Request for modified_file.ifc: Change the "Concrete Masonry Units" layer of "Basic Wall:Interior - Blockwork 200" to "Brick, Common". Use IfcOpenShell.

First a look at what the model holds.

```python
import ifcopenshell
import ifcopenshell.util.element

model = ifcopenshell.open("modified_file.ifc")
print(model.schema)
for layer_set in model.by_type("IfcMaterialLayerSet"):
    if layer_set.LayerSetName == "Basic Wall:Interior - Blockwork 200":
        for layer in layer_set.MaterialLayers:
            print(layer.id(), layer.Material and layer.Material.Name, layer.LayerThickness, sep=" | ")
        print(len(ifcopenshell.util.element.get_elements_by_material(model, layer_set)), "elements and types use it")
print(sorted(m.Name for m in model.by_type("IfcMaterial") if m.Name)[:60])
```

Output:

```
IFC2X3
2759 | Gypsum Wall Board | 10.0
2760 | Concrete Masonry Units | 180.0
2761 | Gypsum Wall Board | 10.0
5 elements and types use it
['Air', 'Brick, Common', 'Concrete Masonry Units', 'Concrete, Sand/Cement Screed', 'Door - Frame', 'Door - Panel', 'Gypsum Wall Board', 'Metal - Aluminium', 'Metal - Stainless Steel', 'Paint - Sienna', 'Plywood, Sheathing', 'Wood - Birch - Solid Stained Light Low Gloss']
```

```python
import ifcopenshell
import ifcopenshell.api.material

model = ifcopenshell.open("modified_file.ifc")

layer_set = next(s for s in model.by_type("IfcMaterialLayerSet") if s.LayerSetName == "Basic Wall:Interior - Blockwork 200")
layer = next(l for l in layer_set.MaterialLayers if l.Material and l.Material.Name == "Concrete Masonry Units")
material = next(m for m in model.by_type("IfcMaterial") if m.Name == "Brick, Common")

# Point this one layer at the other material; renaming the old one would change it everywhere.
ifcopenshell.api.material.edit_layer(model, layer=layer, attributes={}, material=material)

print([l.Material.Name if l.Material else None for l in layer_set.MaterialLayers])

model.write("modified_file_v2.ifc")
```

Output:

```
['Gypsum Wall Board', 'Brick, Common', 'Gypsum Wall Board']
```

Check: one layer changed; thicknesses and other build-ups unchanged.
